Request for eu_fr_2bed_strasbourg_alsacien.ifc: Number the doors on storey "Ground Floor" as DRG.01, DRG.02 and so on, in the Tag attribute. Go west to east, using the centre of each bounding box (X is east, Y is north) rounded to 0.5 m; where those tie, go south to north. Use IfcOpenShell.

First a look at what the model holds.

```python
import ifcopenshell
import ifcopenshell.util.element
import ifcopenshell.util.placement

model = ifcopenshell.open("eu_fr_2bed_strasbourg_alsacien.ifc")
print(model.schema)
storey = next(s for s in model.by_type("IfcBuildingStorey") if s.Name == "Ground Floor")
doors = [e for e in ifcopenshell.util.element.get_decomposition(storey) if e.is_a("IfcDoor")]
for e in sorted(doors, key=lambda e: e.id()):
    origin = ifcopenshell.util.placement.get_local_placement(e.ObjectPlacement)[:3, 3]
    print(e.id(), e.Tag, e.Name, origin.round(2) + 0.0, sep=" | ")
```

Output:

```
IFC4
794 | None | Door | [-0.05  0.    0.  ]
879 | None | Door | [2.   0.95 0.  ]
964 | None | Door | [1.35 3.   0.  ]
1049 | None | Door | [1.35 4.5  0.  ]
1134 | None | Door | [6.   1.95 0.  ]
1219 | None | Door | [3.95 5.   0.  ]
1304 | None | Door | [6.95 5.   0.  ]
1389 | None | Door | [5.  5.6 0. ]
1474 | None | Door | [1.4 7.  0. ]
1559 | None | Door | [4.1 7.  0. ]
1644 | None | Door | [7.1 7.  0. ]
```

```python
import ifcopenshell
import ifcopenshell.geom
import ifcopenshell.util.element
import ifcopenshell.util.shape

model = ifcopenshell.open("eu_fr_2bed_strasbourg_alsacien.ifc")
settings = ifcopenshell.geom.settings()
settings.set("use-world-coords", True)


def centre(element):
    shape = ifcopenshell.geom.create_shape(settings, element)
    return ifcopenshell.util.shape.get_bbox_centroid(shape.geometry)


storey = next(s for s in model.by_type("IfcBuildingStorey") if s.Name == "Ground Floor")
doors = [e for e in ifcopenshell.util.element.get_decomposition(storey) if e.is_a("IfcDoor")]

# Insertion points can sit at a corner or the storey origin, so sort by the geometry (in metres).
centres = {e: centre(e) for e in doors}
doors.sort(key=lambda e: (round(centres[e][0] / 0.5), centres[e][1]))

for i, e in enumerate(doors, start=1):
    number = f"DRG.{i:02d}"
    e.Tag = number
    print(e.id(), number)

model.write("eu_fr_2bed_strasbourg_alsacien-out.ifc")
```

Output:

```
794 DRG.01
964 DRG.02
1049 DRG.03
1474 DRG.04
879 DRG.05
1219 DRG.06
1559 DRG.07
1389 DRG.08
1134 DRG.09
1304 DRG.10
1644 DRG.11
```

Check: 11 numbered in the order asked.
